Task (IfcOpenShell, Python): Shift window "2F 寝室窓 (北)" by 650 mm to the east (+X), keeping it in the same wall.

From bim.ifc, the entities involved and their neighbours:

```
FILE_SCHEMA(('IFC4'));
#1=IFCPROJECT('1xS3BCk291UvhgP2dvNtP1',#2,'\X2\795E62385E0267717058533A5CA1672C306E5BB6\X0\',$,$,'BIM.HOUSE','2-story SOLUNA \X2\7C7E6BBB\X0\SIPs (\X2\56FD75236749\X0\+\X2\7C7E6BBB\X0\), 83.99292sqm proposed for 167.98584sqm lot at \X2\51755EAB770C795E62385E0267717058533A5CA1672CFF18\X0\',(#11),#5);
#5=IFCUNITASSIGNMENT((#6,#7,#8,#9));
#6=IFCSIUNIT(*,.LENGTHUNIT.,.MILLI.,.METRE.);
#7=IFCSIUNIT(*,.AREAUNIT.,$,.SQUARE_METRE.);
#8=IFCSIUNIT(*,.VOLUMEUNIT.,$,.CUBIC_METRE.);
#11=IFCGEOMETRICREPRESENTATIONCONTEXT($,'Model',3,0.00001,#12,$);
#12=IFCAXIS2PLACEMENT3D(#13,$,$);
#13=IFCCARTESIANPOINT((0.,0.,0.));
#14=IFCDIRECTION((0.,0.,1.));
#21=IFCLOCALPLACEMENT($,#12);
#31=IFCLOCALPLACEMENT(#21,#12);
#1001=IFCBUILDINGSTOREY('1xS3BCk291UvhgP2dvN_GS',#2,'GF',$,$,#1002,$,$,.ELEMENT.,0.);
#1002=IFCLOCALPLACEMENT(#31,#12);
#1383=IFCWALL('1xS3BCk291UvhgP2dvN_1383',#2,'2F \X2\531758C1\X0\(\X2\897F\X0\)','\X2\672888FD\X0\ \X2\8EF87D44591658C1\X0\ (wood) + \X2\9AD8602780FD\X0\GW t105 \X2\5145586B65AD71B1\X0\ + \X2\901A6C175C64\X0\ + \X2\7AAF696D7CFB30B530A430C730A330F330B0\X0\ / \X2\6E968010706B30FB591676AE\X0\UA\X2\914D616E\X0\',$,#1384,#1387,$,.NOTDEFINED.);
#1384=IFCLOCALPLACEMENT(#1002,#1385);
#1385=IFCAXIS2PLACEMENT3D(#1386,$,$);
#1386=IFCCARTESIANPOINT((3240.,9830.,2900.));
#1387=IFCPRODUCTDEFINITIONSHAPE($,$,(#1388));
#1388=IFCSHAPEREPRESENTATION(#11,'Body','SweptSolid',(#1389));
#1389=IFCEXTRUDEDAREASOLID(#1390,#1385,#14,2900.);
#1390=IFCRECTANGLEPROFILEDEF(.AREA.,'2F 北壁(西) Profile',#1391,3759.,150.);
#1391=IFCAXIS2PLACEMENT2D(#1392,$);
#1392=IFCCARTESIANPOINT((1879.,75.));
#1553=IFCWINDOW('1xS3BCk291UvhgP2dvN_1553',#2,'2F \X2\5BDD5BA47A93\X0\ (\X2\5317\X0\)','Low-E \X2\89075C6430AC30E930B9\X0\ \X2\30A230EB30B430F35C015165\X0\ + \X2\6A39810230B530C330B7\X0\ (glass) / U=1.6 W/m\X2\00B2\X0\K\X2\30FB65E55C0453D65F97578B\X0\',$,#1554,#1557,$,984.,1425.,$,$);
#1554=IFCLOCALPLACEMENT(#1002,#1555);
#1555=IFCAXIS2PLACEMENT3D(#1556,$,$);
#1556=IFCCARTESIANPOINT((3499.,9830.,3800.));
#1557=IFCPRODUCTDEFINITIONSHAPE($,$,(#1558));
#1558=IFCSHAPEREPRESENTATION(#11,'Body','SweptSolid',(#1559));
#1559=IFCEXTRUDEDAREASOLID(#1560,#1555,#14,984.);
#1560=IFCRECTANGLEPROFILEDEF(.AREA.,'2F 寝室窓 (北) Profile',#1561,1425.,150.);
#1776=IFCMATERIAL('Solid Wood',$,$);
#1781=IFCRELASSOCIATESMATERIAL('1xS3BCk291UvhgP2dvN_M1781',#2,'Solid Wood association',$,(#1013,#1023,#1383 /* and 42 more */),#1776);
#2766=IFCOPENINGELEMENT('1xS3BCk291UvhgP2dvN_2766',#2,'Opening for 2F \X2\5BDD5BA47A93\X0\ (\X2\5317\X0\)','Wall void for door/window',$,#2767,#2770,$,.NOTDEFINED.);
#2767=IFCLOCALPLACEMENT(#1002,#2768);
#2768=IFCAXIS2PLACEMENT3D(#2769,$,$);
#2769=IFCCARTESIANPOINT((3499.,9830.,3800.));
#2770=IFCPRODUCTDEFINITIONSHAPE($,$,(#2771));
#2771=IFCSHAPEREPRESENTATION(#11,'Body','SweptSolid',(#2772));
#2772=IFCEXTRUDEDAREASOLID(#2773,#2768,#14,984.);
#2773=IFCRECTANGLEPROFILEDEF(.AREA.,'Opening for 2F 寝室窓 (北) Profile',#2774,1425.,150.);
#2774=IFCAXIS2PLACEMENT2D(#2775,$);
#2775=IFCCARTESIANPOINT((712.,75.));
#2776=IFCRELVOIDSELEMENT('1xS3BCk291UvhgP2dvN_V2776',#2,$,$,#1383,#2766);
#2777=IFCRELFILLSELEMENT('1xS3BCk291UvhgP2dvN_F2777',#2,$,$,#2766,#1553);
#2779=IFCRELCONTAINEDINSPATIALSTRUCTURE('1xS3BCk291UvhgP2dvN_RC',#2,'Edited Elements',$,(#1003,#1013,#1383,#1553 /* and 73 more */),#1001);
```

```python
import ifcopenshell
import ifcopenshell.api.geometry
import ifcopenshell.util.placement

model = ifcopenshell.open("bim.ifc")

window = model.by_id(1553)
opening = window.FillsVoids[0].RelatingOpeningElement
wall = opening.VoidsElements[0].RelatingBuildingElement

wall_matrix = ifcopenshell.util.placement.get_local_placement(wall.ObjectPlacement)
shift = wall_matrix[:3, 0] * 650.0
before = ifcopenshell.util.placement.get_local_placement(window.ObjectPlacement)[:3, 3].copy()

# The window is not placed relative to its opening, so move both.
for product in (opening, window):
    matrix = ifcopenshell.util.placement.get_local_placement(product.ObjectPlacement)
    matrix[:3, 3] += shift
    ifcopenshell.api.geometry.edit_object_placement(model, product=product, matrix=matrix, is_si=False)

after = ifcopenshell.util.placement.get_local_placement(window.ObjectPlacement)[:3, 3]
print("window moved by", (after - before).round(3) + 0.0)

model.write("bim-out.ifc")
```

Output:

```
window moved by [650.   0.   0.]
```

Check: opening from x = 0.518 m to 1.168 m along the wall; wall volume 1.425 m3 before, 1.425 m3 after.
